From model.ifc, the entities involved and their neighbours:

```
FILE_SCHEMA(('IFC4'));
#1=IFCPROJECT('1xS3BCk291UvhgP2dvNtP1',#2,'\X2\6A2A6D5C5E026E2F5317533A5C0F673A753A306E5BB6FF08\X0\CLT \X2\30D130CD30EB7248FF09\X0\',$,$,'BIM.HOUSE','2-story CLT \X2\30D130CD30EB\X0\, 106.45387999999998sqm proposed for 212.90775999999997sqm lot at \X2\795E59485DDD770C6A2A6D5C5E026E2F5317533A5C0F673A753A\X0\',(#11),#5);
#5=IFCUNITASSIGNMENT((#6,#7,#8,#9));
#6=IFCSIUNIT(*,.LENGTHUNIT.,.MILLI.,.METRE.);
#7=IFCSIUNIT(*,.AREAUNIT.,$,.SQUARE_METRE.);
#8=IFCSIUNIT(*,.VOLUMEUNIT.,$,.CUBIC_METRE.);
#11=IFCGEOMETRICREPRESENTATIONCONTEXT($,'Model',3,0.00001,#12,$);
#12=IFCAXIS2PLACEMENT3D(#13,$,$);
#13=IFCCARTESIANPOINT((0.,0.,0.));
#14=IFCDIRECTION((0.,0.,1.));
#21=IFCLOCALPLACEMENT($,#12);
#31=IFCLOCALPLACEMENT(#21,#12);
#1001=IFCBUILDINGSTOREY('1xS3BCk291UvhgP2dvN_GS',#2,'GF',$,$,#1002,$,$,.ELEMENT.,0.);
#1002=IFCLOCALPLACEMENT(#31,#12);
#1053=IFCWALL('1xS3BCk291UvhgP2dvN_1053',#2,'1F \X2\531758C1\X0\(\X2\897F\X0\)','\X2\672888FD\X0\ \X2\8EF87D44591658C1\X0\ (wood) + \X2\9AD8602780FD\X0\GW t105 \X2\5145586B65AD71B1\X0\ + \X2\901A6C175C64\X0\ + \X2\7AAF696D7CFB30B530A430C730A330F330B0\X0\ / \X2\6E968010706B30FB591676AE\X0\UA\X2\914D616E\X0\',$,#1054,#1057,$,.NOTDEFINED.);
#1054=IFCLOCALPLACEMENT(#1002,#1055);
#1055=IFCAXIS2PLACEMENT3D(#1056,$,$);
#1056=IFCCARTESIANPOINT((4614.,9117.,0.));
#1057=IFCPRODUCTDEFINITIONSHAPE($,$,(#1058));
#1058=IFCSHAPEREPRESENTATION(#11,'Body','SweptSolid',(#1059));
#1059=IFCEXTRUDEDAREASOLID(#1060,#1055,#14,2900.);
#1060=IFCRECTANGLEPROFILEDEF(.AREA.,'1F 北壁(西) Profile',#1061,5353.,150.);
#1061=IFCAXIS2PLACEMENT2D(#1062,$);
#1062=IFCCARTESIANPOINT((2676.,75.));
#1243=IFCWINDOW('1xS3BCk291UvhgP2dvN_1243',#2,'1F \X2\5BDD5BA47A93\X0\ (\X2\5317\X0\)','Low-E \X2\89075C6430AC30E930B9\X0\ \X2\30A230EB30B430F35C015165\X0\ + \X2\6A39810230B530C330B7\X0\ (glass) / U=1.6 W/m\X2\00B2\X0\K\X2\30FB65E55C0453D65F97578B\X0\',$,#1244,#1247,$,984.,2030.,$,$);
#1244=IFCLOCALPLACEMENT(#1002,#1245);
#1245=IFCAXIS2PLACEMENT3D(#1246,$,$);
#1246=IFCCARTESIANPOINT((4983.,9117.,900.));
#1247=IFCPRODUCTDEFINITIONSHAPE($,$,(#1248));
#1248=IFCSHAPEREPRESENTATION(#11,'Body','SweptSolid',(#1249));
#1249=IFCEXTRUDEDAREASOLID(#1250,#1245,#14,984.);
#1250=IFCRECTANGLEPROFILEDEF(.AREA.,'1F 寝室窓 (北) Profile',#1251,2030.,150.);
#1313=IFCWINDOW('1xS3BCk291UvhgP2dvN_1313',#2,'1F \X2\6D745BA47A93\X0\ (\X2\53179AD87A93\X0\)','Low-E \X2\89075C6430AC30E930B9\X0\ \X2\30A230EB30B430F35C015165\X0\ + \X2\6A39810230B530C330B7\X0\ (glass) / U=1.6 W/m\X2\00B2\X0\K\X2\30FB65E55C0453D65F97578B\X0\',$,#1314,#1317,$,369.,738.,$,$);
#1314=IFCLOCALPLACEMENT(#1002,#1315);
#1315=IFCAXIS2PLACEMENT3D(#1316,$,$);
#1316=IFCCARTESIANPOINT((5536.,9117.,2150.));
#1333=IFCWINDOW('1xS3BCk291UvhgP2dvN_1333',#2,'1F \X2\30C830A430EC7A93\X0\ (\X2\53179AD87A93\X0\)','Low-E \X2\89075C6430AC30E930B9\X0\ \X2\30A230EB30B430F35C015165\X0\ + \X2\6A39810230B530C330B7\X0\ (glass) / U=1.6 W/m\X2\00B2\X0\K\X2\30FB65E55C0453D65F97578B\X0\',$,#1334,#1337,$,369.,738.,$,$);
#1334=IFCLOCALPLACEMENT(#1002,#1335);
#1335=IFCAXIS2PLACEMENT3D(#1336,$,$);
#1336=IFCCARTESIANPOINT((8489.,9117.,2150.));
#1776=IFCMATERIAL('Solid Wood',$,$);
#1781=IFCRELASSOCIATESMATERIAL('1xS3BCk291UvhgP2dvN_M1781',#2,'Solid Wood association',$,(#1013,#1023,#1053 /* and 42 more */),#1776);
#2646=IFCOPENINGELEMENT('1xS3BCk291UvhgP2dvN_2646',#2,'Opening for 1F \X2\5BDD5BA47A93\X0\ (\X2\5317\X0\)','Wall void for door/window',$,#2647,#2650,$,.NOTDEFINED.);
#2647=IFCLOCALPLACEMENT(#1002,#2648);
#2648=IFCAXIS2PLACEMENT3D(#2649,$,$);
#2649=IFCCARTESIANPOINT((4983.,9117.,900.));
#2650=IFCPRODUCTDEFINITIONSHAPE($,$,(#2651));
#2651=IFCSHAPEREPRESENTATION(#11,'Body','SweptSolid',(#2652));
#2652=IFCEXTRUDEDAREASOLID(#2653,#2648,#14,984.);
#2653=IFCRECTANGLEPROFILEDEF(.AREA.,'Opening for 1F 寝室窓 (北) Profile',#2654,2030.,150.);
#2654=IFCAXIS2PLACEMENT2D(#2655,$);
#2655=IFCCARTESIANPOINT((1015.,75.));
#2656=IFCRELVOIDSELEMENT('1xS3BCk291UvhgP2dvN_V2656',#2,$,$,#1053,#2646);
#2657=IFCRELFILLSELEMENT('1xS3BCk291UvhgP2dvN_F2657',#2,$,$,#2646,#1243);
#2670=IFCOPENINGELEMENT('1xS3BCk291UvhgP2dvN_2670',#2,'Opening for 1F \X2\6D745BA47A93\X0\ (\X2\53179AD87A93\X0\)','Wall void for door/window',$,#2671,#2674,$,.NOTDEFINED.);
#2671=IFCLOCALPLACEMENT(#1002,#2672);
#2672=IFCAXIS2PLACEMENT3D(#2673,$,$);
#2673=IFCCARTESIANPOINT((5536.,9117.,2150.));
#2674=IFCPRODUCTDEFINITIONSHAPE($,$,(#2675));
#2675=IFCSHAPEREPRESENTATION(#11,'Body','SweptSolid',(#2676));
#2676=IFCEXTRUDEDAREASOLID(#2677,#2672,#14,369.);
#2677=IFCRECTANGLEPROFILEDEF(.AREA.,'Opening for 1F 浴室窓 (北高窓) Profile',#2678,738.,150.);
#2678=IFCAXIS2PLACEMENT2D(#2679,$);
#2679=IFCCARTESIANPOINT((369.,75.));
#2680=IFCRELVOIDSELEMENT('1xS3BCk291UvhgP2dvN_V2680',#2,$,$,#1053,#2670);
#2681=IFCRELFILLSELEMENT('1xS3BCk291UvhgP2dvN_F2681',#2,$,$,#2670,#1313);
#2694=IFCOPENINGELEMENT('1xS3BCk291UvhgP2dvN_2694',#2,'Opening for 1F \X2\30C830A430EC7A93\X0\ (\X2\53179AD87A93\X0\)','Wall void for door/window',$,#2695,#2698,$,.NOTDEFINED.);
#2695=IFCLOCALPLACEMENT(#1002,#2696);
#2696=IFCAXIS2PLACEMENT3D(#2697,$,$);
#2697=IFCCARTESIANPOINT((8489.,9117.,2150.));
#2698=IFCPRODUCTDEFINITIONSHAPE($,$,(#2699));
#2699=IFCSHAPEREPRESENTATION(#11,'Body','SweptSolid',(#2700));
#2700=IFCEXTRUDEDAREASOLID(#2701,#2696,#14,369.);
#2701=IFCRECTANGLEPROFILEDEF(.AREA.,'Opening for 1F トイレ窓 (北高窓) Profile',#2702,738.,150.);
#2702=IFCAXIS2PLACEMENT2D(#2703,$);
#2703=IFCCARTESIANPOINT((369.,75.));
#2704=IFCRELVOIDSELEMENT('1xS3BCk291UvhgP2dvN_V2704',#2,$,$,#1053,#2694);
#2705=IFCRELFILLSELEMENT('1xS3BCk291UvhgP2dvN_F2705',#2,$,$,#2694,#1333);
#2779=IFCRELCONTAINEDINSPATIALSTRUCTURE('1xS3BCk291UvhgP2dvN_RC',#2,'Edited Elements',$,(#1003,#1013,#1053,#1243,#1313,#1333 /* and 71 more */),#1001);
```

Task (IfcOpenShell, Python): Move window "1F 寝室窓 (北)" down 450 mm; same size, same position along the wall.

```python
import numpy as np
import ifcopenshell
import ifcopenshell.api.geometry
import ifcopenshell.util.placement
import ifcopenshell.util.unit

model = ifcopenshell.open("model.ifc")
unit_scale = ifcopenshell.util.unit.calculate_unit_scale(model)

window = model.by_id(1243)
opening = window.FillsVoids[0].RelatingOpeningElement
dz = -0.45 / unit_scale

shift = np.array([0.0, 0.0, dz])
# The window is not placed relative to its opening, so move both.
for product in (opening, window):
    matrix = ifcopenshell.util.placement.get_local_placement(product.ObjectPlacement)
    matrix[:3, 3] += shift
    ifcopenshell.api.geometry.edit_object_placement(model, product=product, matrix=matrix, is_si=False)

print(f"moved by {dz * unit_scale:+.3f} m")

model.write("model_v2.ifc")
```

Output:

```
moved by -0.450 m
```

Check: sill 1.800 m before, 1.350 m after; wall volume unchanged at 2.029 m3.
